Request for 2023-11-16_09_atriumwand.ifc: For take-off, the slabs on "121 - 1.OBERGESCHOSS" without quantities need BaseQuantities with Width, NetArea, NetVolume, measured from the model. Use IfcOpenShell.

First a look at what the model holds.

```python
import ifcopenshell
import ifcopenshell.util.element
import ifcopenshell.util.unit

model = ifcopenshell.open("2023-11-16_09_atriumwand.ifc")
print(model.schema)
for unit_type in ("LENGTHUNIT", "AREAUNIT", "VOLUMEUNIT"):
    print(unit_type, ifcopenshell.util.unit.calculate_unit_scale(model, unit_type))
storey = next(s for s in model.by_type("IfcBuildingStorey") if s.Name == "121 - 1.OBERGESCHOSS")
slabs = [e for e in ifcopenshell.util.element.get_decomposition(storey) if e.is_a("IfcSlab")]
for e in sorted(slabs, key=lambda e: e.id()):
    print(e.id(), e.is_a(), e.Name, list(ifcopenshell.util.element.get_psets(e, qtos_only=True)), sep=" | ")
```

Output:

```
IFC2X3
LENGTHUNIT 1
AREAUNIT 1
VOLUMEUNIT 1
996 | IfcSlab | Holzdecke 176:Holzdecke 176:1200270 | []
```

```python
import ifcopenshell
import ifcopenshell.api.pset
import ifcopenshell.geom
import ifcopenshell.util.element
import ifcopenshell.util.shape
import ifcopenshell.util.unit

model = ifcopenshell.open("2023-11-16_09_atriumwand.ifc")
unit_scale = ifcopenshell.util.unit.calculate_unit_scale(model)
area_scale = ifcopenshell.util.unit.calculate_unit_scale(model, "AREAUNIT")
volume_scale = ifcopenshell.util.unit.calculate_unit_scale(model, "VOLUMEUNIT")
settings = ifcopenshell.geom.settings()

storey = next(s for s in model.by_type("IfcBuildingStorey") if s.Name == "121 - 1.OBERGESCHOSS")
slabs = [e for e in ifcopenshell.util.element.get_decomposition(storey) if e.is_a("IfcSlab")]

for e in sorted(slabs, key=lambda e: e.id()):
    if ifcopenshell.util.element.get_psets(e, qtos_only=True, should_inherit=False):
        continue
    # Geometry comes back in metres, in the element's own axes.
    shape = ifcopenshell.geom.create_shape(settings, e)
    values = {
        "Width": ifcopenshell.util.shape.get_z(shape.geometry) / unit_scale,
        "NetArea": ifcopenshell.util.shape.get_footprint_area(shape.geometry) / area_scale,
        "NetVolume": ifcopenshell.util.shape.get_volume(shape.geometry) / volume_scale,
    }
    qto = ifcopenshell.api.pset.add_qto(model, product=e, name="BaseQuantities")
    ifcopenshell.api.pset.edit_qto(model, qto=qto, properties=values)
    print(e.id(), {k: round(v, 3) for k, v in values.items()})

model.write("2023-11-16_09_atriumwand_edited.ifc")
```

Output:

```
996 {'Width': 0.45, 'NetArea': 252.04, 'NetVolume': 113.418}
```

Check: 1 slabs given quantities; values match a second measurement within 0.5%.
